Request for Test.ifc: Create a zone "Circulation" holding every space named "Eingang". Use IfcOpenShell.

First a look at what the model holds.

```python
import ifcopenshell

model = ifcopenshell.open("Test.ifc")
print(model.schema)
seen = {}
for space in model.by_type("IfcSpace"):
    seen[space.LongName] = seen.get(space.LongName, 0) + 1
for name, count in sorted(seen.items(), key=str):
    print(count, "x", name)
print("zones:", [z.Name for z in model.by_type("IfcZone")][:20])
```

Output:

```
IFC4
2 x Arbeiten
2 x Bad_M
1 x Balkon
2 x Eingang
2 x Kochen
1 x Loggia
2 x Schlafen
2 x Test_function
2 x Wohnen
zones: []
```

```python
import ifcopenshell
import ifcopenshell.api.group
import ifcopenshell.api.root

model = ifcopenshell.open("Test.ifc")

names = {"Eingang"}
spaces = [s for s in model.by_type("IfcSpace") if s.LongName in names]

zone = ifcopenshell.api.root.create_entity(model, ifc_class="IfcZone", name="Circulation")
ifcopenshell.api.group.assign_group(model, products=spaces, group=zone)
print(len(spaces), "spaces in", zone.Name)

model.write("Test_updated.ifc")
```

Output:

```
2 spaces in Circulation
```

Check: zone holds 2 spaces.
